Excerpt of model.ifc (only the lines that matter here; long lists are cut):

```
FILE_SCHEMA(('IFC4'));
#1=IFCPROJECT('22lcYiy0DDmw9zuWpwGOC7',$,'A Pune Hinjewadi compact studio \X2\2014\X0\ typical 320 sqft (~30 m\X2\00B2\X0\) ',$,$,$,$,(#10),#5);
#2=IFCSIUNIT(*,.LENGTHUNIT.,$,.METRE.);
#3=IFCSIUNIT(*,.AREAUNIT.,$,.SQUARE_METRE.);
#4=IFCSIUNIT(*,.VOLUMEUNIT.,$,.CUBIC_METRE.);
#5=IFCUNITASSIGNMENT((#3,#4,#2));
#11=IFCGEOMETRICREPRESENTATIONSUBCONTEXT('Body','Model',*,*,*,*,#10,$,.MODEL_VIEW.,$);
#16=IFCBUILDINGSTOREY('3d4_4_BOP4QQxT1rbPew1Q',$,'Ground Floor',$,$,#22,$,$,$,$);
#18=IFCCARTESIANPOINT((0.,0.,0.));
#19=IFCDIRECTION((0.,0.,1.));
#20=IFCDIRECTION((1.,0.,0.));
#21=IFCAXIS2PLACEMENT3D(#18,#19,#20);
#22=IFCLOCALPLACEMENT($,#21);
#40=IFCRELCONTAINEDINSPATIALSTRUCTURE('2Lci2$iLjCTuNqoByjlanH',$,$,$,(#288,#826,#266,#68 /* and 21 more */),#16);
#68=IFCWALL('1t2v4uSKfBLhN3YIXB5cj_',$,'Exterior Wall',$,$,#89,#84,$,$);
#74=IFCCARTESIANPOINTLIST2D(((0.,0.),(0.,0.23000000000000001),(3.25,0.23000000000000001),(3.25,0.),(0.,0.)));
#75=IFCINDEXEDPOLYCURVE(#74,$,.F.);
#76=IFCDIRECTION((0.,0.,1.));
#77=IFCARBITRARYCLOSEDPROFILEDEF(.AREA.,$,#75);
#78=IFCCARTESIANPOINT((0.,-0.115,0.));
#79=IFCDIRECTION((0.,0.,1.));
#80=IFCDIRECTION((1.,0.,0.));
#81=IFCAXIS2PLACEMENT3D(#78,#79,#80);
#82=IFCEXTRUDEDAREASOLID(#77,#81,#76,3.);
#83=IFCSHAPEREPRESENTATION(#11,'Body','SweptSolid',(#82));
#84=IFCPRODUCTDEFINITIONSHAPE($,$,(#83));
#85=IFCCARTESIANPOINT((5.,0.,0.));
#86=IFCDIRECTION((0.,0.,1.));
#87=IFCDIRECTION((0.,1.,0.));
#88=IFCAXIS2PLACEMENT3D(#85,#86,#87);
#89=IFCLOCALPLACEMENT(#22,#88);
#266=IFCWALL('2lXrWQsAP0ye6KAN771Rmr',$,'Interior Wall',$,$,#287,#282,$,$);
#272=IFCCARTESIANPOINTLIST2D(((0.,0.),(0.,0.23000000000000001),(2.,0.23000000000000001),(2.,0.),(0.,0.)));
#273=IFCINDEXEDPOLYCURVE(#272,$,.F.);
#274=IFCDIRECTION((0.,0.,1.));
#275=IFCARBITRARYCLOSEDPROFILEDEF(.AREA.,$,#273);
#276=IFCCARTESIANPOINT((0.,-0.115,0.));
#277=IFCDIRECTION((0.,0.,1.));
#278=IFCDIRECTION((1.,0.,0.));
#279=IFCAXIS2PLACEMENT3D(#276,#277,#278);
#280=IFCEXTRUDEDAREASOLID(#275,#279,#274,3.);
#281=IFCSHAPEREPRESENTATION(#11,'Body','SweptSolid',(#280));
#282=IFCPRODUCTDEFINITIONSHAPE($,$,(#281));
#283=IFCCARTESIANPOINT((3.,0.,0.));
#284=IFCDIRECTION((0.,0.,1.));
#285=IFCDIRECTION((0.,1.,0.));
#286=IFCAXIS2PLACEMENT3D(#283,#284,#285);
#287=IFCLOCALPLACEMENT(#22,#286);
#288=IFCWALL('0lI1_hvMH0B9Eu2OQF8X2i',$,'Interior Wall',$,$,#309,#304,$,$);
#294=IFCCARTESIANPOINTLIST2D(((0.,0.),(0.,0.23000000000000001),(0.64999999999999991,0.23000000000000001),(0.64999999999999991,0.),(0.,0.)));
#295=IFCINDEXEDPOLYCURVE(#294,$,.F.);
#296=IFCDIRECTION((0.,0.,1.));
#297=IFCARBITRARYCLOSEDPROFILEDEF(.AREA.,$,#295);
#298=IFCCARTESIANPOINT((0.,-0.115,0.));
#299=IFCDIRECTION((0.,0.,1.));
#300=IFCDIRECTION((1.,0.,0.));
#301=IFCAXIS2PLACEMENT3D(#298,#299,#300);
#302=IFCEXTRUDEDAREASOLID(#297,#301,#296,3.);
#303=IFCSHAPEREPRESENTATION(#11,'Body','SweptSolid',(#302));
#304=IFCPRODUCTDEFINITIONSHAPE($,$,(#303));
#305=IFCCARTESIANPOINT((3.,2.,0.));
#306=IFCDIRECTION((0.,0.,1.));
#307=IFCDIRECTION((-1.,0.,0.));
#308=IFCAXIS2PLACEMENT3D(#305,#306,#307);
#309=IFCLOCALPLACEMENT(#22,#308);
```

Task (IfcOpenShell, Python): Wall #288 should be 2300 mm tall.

```python
import ifcopenshell
import ifcopenshell.geom
import ifcopenshell.util.representation
import ifcopenshell.util.shape

model = ifcopenshell.open("model.ifc")
settings = ifcopenshell.geom.settings()


def volume(element):
    """Net volume in cubic metres, openings subtracted."""
    shape = ifcopenshell.geom.create_shape(settings, element)
    return ifcopenshell.util.shape.get_volume(shape.geometry)


wall = model.by_id(288)
before = volume(wall)

body = ifcopenshell.util.representation.get_representation(wall, "Model", "Body")
solid = body.Items[0]
old_height = solid.Depth
solid.Depth = 2.3
after = volume(wall)

print(f"height {old_height:g} -> {solid.Depth:g}, volume {before:.3f} -> {after:.3f} m3")

model.write("model_v2.ifc")
```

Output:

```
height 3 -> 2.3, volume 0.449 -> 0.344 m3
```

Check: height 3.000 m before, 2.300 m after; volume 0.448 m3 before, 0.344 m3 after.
